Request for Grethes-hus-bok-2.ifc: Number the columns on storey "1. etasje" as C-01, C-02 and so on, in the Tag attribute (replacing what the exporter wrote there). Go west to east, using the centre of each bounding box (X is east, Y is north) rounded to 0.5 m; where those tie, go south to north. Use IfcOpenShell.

First a look at what the model holds.

```python
import ifcopenshell
import ifcopenshell.util.element
import ifcopenshell.util.placement

model = ifcopenshell.open("Grethes-hus-bok-2.ifc")
print(model.schema)
storey = next(s for s in model.by_type("IfcBuildingStorey") if s.Name == "1. etasje")
columns = [e for e in ifcopenshell.util.element.get_decomposition(storey) if e.is_a("IfcColumn")]
for e in sorted(columns, key=lambda e: e.id()):
    origin = ifcopenshell.util.placement.get_local_placement(e.ObjectPlacement)[:3, 3]
    print(e.id(), e.Tag, e.Name, origin.round(2) + 0.0, sep=" | ")
```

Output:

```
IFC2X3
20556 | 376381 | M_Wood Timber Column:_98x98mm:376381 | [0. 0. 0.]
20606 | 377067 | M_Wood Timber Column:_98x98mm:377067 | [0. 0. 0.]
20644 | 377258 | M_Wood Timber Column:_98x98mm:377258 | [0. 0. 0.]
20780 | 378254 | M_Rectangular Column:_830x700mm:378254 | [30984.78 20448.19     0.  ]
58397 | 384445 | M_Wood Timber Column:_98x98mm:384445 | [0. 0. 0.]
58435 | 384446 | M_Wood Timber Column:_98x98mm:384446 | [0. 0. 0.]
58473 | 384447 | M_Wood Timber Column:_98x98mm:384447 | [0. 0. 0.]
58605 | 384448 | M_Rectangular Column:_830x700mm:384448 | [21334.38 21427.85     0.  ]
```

```python
import ifcopenshell
import ifcopenshell.geom
import ifcopenshell.util.element
import ifcopenshell.util.shape

model = ifcopenshell.open("Grethes-hus-bok-2.ifc")
settings = ifcopenshell.geom.settings()
settings.set("use-world-coords", True)


def centre(element):
    shape = ifcopenshell.geom.create_shape(settings, element)
    return ifcopenshell.util.shape.get_bbox_centroid(shape.geometry)


storey = next(s for s in model.by_type("IfcBuildingStorey") if s.Name == "1. etasje")
columns = [e for e in ifcopenshell.util.element.get_decomposition(storey) if e.is_a("IfcColumn")]

# Insertion points can sit at a corner or the storey origin, so sort by the geometry (in metres).
centres = {e: centre(e) for e in columns}
columns.sort(key=lambda e: (round(centres[e][0] / 0.5), centres[e][1]))

for i, e in enumerate(columns, start=1):
    number = f"C-{i:02d}"
    e.Tag = number
    print(e.id(), number)

model.write("Grethes-hus-bok-2_updated.ifc")
```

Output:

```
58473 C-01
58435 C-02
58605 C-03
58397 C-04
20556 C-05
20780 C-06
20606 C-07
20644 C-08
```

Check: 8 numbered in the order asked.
